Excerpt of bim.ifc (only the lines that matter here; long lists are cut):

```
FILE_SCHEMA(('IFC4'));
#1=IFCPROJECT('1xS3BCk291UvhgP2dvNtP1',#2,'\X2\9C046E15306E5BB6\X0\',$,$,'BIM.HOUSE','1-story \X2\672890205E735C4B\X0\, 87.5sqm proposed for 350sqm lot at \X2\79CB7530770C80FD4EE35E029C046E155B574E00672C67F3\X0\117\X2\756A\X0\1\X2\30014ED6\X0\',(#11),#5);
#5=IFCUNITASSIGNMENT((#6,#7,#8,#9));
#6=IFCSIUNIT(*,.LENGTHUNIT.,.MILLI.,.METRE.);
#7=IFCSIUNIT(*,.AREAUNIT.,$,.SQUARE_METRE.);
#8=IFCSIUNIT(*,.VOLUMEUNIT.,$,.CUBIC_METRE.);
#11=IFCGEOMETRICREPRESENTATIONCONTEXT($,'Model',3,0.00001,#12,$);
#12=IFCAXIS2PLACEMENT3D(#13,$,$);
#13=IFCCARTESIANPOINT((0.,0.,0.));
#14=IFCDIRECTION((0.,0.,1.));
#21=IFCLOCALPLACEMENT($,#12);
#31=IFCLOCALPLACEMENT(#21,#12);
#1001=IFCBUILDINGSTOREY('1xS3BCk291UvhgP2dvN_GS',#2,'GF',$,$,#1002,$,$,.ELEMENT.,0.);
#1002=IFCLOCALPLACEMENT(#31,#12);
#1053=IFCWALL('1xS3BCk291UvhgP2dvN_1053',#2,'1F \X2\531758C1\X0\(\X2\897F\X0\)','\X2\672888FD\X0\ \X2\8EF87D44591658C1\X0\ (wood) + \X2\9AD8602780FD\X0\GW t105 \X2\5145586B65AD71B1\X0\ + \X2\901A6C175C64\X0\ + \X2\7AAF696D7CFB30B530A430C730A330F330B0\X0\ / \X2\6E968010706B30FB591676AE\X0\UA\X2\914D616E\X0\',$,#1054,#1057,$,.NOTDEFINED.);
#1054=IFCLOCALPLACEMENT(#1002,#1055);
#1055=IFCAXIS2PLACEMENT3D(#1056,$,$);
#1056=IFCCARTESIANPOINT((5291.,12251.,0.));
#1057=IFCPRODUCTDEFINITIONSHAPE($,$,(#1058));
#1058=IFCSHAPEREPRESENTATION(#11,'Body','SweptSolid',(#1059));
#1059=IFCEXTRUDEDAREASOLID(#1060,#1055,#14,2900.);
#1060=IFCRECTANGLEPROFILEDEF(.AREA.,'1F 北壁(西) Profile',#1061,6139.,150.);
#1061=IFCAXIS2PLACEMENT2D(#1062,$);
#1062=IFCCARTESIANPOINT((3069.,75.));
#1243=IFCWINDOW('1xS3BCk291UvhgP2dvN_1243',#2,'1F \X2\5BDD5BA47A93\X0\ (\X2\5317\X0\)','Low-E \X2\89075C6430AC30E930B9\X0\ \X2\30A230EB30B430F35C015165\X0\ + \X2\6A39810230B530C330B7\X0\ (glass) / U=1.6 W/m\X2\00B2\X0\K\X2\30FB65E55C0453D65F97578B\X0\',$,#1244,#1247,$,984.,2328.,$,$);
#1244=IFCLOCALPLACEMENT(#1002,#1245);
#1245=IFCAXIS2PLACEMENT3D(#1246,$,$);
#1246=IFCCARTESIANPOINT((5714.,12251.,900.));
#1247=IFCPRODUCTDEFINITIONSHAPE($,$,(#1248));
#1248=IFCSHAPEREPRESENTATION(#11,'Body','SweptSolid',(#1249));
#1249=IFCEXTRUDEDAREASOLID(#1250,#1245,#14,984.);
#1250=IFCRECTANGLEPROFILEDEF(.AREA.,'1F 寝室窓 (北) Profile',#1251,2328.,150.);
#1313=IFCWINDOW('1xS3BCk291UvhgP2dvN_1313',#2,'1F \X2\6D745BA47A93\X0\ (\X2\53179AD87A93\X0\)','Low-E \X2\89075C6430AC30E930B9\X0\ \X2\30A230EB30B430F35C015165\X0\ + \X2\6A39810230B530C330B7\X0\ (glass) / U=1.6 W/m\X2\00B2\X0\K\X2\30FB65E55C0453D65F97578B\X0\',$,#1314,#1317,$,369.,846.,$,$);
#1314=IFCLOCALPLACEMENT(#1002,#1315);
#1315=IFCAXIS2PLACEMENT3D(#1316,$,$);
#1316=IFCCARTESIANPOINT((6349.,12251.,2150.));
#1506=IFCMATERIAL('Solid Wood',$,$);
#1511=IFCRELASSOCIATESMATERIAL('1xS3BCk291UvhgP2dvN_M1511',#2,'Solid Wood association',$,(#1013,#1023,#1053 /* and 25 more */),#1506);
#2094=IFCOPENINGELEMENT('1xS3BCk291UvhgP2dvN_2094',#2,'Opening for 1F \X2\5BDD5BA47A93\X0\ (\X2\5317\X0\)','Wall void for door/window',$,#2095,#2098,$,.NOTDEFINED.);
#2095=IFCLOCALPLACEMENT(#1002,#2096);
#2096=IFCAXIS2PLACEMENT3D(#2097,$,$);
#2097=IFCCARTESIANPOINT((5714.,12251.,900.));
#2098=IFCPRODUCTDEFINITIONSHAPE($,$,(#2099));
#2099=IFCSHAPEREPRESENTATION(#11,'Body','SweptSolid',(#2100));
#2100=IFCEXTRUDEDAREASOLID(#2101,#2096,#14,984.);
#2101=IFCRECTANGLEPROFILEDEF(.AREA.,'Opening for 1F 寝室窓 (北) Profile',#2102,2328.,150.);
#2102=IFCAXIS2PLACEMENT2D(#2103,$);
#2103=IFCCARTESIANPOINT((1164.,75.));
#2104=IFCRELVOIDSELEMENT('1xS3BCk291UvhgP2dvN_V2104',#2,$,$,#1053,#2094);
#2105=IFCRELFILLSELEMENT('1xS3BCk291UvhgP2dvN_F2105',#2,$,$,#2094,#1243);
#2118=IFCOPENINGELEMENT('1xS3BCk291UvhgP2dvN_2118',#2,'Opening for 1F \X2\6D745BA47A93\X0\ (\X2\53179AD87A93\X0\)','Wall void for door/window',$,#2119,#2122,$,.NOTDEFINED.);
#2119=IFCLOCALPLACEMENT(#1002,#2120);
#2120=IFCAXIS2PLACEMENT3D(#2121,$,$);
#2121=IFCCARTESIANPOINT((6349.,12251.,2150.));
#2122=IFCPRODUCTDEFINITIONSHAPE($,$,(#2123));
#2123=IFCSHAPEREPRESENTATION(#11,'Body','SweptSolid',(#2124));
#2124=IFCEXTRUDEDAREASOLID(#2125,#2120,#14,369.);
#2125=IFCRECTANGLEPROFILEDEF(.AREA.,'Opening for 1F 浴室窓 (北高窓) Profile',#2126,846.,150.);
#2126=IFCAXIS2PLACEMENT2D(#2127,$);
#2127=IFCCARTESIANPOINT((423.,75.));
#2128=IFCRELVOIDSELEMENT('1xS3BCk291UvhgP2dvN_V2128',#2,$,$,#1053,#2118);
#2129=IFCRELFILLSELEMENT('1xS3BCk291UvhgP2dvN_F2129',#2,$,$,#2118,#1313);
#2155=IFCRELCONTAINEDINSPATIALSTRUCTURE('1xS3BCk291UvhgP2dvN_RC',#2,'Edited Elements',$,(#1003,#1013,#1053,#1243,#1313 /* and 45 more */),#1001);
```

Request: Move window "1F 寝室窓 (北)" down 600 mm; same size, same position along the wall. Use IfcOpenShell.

```python
import numpy as np
import ifcopenshell
import ifcopenshell.api.geometry
import ifcopenshell.util.placement
import ifcopenshell.util.unit

model = ifcopenshell.open("bim.ifc")
unit_scale = ifcopenshell.util.unit.calculate_unit_scale(model)

window = model.by_guid("1xS3BCk291UvhgP2dvN_1243")
opening = window.FillsVoids[0].RelatingOpeningElement
dz = -600.0

shift = np.array([0.0, 0.0, dz])
# The window is not placed relative to its opening, so move both.
for product in (opening, window):
    matrix = ifcopenshell.util.placement.get_local_placement(product.ObjectPlacement)
    matrix[:3, 3] += shift
    ifcopenshell.api.geometry.edit_object_placement(model, product=product, matrix=matrix, is_si=False)

print(f"moved by {dz * unit_scale:+.3f} m")

model.write("bim_rev.ifc")
```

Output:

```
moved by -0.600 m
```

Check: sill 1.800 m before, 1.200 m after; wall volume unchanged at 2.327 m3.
